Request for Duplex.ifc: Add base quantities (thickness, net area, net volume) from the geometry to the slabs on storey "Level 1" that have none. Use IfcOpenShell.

First a look at what the model holds.

```python
import ifcopenshell
import ifcopenshell.util.element
import ifcopenshell.util.unit

model = ifcopenshell.open("Duplex.ifc")
print(model.schema)
for unit_type in ("LENGTHUNIT", "AREAUNIT", "VOLUMEUNIT"):
    print(unit_type, ifcopenshell.util.unit.calculate_unit_scale(model, unit_type))
storey = next(s for s in model.by_type("IfcBuildingStorey") if s.Name == "Level 1")
slabs = [e for e in ifcopenshell.util.element.get_decomposition(storey) if e.is_a("IfcSlab")]
for e in sorted(slabs, key=lambda e: e.id()):
    print(e.id(), e.is_a(), e.Name, list(ifcopenshell.util.element.get_psets(e, qtos_only=True)), sep=" | ")
```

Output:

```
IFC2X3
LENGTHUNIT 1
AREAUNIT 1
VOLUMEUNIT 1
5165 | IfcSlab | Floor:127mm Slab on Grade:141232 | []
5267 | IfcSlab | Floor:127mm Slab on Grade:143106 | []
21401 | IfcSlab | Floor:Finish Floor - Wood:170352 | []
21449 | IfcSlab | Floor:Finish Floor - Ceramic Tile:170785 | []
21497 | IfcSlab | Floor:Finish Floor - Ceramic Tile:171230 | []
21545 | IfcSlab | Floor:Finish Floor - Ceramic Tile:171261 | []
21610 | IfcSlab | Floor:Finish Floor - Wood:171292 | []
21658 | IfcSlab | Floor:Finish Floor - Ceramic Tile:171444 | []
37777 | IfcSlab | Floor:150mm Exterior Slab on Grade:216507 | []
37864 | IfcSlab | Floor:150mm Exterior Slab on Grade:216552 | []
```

```python
import ifcopenshell
import ifcopenshell.api.pset
import ifcopenshell.geom
import ifcopenshell.util.element
import ifcopenshell.util.shape
import ifcopenshell.util.unit

model = ifcopenshell.open("Duplex.ifc")
unit_scale = ifcopenshell.util.unit.calculate_unit_scale(model)
area_scale = ifcopenshell.util.unit.calculate_unit_scale(model, "AREAUNIT")
volume_scale = ifcopenshell.util.unit.calculate_unit_scale(model, "VOLUMEUNIT")
settings = ifcopenshell.geom.settings()

storey = next(s for s in model.by_type("IfcBuildingStorey") if s.Name == "Level 1")
slabs = [e for e in ifcopenshell.util.element.get_decomposition(storey) if e.is_a("IfcSlab")]

for e in sorted(slabs, key=lambda e: e.id()):
    if ifcopenshell.util.element.get_psets(e, qtos_only=True, should_inherit=False):
        continue
    # Geometry comes back in metres, in the element's own axes.
    shape = ifcopenshell.geom.create_shape(settings, e)
    values = {
        "Width": ifcopenshell.util.shape.get_z(shape.geometry) / unit_scale,
        "NetArea": ifcopenshell.util.shape.get_footprint_area(shape.geometry) / area_scale,
        "NetVolume": ifcopenshell.util.shape.get_volume(shape.geometry) / volume_scale,
    }
    qto = ifcopenshell.api.pset.add_qto(model, product=e, name="BaseQuantities")
    ifcopenshell.api.pset.edit_qto(model, qto=qto, properties=values)
    print(e.id(), {k: round(v, 3) for k, v in values.items()})

model.write("Duplex_v2.ifc")
```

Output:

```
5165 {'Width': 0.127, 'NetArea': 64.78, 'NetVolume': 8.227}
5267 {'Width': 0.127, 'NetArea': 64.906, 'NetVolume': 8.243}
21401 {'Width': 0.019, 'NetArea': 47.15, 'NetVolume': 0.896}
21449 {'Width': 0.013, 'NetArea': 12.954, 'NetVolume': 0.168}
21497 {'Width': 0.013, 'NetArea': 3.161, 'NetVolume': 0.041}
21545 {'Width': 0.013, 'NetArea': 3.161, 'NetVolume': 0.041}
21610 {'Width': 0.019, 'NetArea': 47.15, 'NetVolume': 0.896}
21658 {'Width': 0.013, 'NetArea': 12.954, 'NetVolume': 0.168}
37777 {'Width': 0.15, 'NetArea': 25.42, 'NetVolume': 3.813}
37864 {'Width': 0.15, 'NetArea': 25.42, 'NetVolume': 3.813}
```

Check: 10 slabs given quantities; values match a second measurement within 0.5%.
